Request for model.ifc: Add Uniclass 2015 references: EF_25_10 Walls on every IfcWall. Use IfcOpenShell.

First a look at what the model holds.

```python
import ifcopenshell

model = ifcopenshell.open("model.ifc")
print(model.schema)
print("classifications:", [c.Name for c in model.by_type("IfcClassification")])
for ifc_class in ("IfcDoor", "IfcRoof", "IfcStair", "IfcWall", "IfcWindow"):
    print(ifc_class, len(model.by_type(ifc_class)))
```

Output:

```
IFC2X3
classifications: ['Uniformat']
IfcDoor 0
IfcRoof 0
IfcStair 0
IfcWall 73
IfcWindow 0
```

```python
import ifcopenshell
import ifcopenshell.api.classification

model = ifcopenshell.open("model.ifc")

# IFC2X3 requires Source and Edition and has no link from the project to the system.
system = model.create_entity("IfcClassification", Source="NBS", Edition="2015", Name="Uniclass 2015")

codes = {
    "IfcWall": ("EF_25_10", "Walls"),
}
for ifc_class, (code, name) in codes.items():
    products = model.by_type(ifc_class)
    ifcopenshell.api.classification.add_reference(
        model, products=products, classification=system, identification=code, name=name
    )
    print(code, len(products))

model.write("model_rev.ifc")
```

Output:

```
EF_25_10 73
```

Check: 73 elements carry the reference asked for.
